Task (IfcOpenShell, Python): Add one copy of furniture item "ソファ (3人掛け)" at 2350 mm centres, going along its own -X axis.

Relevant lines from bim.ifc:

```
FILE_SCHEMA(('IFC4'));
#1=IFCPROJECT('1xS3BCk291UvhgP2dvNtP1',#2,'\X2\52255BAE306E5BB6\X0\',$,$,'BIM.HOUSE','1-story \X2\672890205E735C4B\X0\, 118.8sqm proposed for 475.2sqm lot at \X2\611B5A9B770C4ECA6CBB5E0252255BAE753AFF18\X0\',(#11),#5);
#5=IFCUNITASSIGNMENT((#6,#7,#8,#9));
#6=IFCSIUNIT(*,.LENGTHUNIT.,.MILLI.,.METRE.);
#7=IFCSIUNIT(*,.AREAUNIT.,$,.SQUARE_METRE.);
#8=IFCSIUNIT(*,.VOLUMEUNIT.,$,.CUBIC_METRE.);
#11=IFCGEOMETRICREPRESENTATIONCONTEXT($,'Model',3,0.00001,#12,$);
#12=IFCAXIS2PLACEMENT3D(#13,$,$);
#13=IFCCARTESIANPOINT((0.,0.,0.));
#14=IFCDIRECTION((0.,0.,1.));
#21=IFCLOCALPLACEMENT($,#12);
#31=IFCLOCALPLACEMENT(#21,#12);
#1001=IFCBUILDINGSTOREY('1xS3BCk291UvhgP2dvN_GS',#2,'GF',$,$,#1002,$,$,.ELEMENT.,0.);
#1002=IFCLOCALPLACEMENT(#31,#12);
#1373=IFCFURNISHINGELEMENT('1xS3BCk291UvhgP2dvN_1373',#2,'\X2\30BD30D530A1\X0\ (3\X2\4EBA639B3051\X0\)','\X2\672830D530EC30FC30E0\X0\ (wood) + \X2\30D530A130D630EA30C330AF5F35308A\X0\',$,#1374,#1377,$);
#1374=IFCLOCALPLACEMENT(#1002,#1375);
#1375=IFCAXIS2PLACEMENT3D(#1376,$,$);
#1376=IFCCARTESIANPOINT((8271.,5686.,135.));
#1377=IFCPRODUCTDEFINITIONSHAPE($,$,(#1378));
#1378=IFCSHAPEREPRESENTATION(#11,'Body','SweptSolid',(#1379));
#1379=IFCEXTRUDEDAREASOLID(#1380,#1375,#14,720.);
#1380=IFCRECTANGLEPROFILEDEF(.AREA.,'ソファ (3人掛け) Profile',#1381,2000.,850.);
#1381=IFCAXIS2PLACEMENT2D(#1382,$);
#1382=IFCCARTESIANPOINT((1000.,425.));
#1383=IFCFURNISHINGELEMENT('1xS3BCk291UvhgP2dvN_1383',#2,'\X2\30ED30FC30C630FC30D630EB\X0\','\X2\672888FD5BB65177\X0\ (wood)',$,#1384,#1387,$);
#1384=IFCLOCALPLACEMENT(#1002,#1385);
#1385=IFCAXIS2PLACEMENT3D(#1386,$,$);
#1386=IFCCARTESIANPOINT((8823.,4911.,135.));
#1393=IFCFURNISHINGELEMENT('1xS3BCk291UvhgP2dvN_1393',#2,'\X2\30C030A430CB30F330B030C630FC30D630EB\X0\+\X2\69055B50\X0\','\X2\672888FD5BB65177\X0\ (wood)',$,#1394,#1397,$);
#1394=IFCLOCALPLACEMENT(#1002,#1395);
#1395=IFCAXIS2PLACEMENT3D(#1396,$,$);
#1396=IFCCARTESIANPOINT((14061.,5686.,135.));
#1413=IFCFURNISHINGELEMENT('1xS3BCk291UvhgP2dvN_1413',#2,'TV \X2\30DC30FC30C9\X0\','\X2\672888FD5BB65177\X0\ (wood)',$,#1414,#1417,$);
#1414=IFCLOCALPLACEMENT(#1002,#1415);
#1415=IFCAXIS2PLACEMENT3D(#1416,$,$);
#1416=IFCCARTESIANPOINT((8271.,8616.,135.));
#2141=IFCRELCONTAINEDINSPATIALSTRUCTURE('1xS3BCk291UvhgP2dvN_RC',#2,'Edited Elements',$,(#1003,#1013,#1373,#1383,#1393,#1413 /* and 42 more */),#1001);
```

```python
import ifcopenshell
import ifcopenshell.api.geometry
import ifcopenshell.api.root
import ifcopenshell.util.element
import ifcopenshell.util.placement
import ifcopenshell.util.unit

model = ifcopenshell.open("bim.ifc")
unit_scale = ifcopenshell.util.unit.calculate_unit_scale(model)


def reuse_history(source, copy):
    """copy_class also copies each property set's owner history, people and application; keep the originals."""
    for rel in copy.IsDefinedBy:
        if rel.is_a("IfcRelDefinesByProperties") and (history := rel.RelatingPropertyDefinition.OwnerHistory):
            rel.RelatingPropertyDefinition.OwnerHistory = source.OwnerHistory
            ifcopenshell.util.element.remove_deep2(model, history)


source = model.by_guid("1xS3BCk291UvhgP2dvN_1373")
base = ifcopenshell.util.placement.get_local_placement(source.ObjectPlacement)
step = -base[:3, 0] * 2.35 / unit_scale

for i in range(1, 2):
    copy = ifcopenshell.api.root.copy_class(model, product=source)
    copy.Representation = ifcopenshell.util.element.copy_deep(
        model, source.Representation, exclude=["IfcGeometricRepresentationContext", "IfcRepresentationMap"]
    )
    reuse_history(source, copy)
    matrix = base.copy()
    matrix[:3, 3] += i * step
    print("added at", matrix[:3, 3].round(3) + 0.0)
    ifcopenshell.api.geometry.edit_object_placement(model, product=copy, matrix=matrix, is_si=False)

model.write("bim_rev.ifc")
```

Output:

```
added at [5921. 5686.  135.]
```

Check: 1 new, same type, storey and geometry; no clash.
